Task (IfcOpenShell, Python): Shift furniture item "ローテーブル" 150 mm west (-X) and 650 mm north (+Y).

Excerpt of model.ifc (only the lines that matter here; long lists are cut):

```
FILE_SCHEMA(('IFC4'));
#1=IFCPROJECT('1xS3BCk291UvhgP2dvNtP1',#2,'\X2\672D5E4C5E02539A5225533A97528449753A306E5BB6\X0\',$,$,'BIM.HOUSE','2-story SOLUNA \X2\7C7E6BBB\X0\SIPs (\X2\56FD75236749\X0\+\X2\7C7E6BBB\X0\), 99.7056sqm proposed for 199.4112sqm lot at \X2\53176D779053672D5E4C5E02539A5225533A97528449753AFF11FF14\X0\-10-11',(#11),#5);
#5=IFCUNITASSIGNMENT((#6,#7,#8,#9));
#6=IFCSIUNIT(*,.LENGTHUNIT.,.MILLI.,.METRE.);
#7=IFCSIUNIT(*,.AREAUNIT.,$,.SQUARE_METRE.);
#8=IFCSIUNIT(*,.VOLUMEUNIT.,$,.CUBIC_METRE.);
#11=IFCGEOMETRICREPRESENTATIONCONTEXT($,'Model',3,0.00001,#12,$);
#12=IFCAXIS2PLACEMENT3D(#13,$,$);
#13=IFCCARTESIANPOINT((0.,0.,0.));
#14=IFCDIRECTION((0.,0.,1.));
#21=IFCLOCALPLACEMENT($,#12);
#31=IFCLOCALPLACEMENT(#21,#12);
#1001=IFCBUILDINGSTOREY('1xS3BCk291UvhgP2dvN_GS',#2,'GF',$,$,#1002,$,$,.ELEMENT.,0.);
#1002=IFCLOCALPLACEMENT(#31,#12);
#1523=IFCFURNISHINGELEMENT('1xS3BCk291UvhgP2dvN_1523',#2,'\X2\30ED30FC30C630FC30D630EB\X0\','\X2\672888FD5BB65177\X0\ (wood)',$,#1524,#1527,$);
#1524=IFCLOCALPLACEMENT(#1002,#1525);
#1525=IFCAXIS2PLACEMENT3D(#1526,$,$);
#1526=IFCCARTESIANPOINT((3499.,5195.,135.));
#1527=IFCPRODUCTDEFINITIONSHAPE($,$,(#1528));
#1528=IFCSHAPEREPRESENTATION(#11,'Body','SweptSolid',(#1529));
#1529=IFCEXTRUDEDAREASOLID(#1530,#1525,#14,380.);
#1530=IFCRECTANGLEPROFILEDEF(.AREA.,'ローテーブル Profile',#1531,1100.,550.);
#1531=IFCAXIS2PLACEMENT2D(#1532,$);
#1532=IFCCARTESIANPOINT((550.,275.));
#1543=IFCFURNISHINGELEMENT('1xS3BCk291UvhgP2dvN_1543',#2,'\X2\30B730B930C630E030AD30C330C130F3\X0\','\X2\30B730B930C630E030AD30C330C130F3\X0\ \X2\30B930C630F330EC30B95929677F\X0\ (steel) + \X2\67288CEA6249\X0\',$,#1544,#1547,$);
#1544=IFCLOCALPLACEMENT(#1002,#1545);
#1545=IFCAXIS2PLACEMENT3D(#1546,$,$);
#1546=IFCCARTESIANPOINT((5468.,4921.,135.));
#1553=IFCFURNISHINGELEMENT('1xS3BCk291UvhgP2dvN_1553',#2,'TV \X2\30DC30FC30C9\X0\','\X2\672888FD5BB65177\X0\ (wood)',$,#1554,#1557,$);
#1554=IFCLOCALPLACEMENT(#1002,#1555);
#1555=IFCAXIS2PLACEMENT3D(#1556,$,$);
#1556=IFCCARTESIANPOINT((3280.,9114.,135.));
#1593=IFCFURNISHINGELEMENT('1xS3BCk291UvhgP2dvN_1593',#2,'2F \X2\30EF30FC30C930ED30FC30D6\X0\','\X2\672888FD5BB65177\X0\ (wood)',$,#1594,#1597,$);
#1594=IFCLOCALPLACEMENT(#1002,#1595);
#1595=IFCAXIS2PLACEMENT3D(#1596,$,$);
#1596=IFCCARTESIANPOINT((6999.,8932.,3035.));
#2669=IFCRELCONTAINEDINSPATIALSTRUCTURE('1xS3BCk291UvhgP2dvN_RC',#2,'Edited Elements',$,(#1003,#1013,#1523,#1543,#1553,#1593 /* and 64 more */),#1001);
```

```python
import ifcopenshell
import ifcopenshell.api.geometry
import ifcopenshell.util.placement

model = ifcopenshell.open("model.ifc")

item = model.by_guid("1xS3BCk291UvhgP2dvN_1523")
matrix = ifcopenshell.util.placement.get_local_placement(item.ObjectPlacement)
matrix[0, 3] -= 150.0
matrix[1, 3] += 650.0
ifcopenshell.api.geometry.edit_object_placement(model, product=item, matrix=matrix, is_si=False)

print(ifcopenshell.util.placement.get_local_placement(item.ObjectPlacement).round(3) + 0.0)

model.write("model-out.ifc")
```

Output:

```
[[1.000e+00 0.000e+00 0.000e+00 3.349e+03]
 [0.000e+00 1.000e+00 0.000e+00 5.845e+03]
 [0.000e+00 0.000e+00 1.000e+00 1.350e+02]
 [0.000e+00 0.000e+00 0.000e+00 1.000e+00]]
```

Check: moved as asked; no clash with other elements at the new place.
